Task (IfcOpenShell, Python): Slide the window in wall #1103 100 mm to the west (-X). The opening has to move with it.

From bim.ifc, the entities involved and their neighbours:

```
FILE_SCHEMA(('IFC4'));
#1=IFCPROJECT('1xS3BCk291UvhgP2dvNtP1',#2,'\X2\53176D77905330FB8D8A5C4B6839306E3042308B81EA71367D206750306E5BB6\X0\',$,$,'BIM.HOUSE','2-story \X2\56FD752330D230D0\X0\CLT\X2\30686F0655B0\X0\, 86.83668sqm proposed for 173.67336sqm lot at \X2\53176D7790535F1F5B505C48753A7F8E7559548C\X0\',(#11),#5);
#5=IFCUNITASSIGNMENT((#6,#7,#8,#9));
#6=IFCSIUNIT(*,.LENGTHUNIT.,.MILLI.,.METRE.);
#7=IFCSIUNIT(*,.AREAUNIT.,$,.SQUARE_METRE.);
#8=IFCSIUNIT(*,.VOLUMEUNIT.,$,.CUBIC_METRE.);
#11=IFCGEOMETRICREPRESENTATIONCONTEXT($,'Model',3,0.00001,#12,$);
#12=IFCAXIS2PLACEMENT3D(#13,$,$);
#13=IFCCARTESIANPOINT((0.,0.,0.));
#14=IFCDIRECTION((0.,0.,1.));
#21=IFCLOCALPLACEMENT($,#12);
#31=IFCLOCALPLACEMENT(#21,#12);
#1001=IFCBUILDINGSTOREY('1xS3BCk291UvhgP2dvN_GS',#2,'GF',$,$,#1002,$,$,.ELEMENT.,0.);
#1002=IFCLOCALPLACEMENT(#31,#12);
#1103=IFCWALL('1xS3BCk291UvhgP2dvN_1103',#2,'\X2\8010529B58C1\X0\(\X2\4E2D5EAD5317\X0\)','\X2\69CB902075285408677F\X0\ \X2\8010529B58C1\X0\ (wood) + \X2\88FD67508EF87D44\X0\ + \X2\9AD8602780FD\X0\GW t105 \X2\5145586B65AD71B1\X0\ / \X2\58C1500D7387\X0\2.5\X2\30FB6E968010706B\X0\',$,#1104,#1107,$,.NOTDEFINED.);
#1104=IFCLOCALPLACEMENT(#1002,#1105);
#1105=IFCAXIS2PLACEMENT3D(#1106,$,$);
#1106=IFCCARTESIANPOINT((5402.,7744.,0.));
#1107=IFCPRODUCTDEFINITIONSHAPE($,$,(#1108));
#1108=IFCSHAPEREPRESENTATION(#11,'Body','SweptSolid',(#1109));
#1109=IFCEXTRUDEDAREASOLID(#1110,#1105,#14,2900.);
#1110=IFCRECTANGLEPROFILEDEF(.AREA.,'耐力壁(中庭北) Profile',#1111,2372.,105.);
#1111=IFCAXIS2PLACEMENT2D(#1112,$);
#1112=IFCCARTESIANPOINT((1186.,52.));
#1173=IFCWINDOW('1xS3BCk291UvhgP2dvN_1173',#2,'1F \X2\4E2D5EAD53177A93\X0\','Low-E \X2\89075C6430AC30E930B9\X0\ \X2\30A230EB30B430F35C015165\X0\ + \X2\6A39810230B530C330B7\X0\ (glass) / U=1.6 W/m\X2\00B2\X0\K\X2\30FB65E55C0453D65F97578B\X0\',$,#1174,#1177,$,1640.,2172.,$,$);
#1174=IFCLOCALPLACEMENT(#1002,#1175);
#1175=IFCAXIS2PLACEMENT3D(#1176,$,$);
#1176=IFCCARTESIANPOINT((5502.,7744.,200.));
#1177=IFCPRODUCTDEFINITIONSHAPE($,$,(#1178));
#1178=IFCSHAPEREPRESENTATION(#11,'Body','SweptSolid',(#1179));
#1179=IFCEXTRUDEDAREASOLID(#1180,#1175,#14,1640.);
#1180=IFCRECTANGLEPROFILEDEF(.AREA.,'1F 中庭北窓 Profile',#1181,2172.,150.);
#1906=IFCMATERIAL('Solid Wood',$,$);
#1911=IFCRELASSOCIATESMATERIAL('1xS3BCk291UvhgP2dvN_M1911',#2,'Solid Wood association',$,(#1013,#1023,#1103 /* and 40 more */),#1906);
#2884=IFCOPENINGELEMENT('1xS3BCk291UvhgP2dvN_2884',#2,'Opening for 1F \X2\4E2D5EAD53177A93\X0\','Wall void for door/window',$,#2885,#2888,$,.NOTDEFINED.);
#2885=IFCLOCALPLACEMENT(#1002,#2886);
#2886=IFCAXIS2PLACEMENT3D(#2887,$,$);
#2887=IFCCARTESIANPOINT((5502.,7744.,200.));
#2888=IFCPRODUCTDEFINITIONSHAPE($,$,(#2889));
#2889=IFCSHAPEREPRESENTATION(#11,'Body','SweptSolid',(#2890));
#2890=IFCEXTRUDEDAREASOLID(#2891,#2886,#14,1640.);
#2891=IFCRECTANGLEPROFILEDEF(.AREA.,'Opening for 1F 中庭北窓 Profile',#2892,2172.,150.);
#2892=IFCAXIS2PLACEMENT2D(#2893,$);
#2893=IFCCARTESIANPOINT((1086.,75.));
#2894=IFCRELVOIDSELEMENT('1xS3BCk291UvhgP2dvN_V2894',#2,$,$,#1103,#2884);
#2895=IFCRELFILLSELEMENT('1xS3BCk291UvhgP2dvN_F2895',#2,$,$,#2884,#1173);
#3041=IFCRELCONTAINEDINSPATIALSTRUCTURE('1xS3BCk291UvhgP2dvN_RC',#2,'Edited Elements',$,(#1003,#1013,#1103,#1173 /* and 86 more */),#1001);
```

```python
import ifcopenshell
import ifcopenshell.api.geometry
import ifcopenshell.util.placement

model = ifcopenshell.open("bim.ifc")

window = model.by_guid("1xS3BCk291UvhgP2dvN_1173")
opening = window.FillsVoids[0].RelatingOpeningElement
wall = opening.VoidsElements[0].RelatingBuildingElement

wall_matrix = ifcopenshell.util.placement.get_local_placement(wall.ObjectPlacement)
shift = wall_matrix[:3, 0] * -100.0
before = ifcopenshell.util.placement.get_local_placement(window.ObjectPlacement)[:3, 3].copy()

# The window is not placed relative to its opening, so move both.
for product in (opening, window):
    matrix = ifcopenshell.util.placement.get_local_placement(product.ObjectPlacement)
    matrix[:3, 3] += shift
    ifcopenshell.api.geometry.edit_object_placement(model, product=product, matrix=matrix, is_si=False)

after = ifcopenshell.util.placement.get_local_placement(window.ObjectPlacement)[:3, 3]
print("window moved by", (after - before).round(3) + 0.0)

model.write("bim_rev.ifc")
```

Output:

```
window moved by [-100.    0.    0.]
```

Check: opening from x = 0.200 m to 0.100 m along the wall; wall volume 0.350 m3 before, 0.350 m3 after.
